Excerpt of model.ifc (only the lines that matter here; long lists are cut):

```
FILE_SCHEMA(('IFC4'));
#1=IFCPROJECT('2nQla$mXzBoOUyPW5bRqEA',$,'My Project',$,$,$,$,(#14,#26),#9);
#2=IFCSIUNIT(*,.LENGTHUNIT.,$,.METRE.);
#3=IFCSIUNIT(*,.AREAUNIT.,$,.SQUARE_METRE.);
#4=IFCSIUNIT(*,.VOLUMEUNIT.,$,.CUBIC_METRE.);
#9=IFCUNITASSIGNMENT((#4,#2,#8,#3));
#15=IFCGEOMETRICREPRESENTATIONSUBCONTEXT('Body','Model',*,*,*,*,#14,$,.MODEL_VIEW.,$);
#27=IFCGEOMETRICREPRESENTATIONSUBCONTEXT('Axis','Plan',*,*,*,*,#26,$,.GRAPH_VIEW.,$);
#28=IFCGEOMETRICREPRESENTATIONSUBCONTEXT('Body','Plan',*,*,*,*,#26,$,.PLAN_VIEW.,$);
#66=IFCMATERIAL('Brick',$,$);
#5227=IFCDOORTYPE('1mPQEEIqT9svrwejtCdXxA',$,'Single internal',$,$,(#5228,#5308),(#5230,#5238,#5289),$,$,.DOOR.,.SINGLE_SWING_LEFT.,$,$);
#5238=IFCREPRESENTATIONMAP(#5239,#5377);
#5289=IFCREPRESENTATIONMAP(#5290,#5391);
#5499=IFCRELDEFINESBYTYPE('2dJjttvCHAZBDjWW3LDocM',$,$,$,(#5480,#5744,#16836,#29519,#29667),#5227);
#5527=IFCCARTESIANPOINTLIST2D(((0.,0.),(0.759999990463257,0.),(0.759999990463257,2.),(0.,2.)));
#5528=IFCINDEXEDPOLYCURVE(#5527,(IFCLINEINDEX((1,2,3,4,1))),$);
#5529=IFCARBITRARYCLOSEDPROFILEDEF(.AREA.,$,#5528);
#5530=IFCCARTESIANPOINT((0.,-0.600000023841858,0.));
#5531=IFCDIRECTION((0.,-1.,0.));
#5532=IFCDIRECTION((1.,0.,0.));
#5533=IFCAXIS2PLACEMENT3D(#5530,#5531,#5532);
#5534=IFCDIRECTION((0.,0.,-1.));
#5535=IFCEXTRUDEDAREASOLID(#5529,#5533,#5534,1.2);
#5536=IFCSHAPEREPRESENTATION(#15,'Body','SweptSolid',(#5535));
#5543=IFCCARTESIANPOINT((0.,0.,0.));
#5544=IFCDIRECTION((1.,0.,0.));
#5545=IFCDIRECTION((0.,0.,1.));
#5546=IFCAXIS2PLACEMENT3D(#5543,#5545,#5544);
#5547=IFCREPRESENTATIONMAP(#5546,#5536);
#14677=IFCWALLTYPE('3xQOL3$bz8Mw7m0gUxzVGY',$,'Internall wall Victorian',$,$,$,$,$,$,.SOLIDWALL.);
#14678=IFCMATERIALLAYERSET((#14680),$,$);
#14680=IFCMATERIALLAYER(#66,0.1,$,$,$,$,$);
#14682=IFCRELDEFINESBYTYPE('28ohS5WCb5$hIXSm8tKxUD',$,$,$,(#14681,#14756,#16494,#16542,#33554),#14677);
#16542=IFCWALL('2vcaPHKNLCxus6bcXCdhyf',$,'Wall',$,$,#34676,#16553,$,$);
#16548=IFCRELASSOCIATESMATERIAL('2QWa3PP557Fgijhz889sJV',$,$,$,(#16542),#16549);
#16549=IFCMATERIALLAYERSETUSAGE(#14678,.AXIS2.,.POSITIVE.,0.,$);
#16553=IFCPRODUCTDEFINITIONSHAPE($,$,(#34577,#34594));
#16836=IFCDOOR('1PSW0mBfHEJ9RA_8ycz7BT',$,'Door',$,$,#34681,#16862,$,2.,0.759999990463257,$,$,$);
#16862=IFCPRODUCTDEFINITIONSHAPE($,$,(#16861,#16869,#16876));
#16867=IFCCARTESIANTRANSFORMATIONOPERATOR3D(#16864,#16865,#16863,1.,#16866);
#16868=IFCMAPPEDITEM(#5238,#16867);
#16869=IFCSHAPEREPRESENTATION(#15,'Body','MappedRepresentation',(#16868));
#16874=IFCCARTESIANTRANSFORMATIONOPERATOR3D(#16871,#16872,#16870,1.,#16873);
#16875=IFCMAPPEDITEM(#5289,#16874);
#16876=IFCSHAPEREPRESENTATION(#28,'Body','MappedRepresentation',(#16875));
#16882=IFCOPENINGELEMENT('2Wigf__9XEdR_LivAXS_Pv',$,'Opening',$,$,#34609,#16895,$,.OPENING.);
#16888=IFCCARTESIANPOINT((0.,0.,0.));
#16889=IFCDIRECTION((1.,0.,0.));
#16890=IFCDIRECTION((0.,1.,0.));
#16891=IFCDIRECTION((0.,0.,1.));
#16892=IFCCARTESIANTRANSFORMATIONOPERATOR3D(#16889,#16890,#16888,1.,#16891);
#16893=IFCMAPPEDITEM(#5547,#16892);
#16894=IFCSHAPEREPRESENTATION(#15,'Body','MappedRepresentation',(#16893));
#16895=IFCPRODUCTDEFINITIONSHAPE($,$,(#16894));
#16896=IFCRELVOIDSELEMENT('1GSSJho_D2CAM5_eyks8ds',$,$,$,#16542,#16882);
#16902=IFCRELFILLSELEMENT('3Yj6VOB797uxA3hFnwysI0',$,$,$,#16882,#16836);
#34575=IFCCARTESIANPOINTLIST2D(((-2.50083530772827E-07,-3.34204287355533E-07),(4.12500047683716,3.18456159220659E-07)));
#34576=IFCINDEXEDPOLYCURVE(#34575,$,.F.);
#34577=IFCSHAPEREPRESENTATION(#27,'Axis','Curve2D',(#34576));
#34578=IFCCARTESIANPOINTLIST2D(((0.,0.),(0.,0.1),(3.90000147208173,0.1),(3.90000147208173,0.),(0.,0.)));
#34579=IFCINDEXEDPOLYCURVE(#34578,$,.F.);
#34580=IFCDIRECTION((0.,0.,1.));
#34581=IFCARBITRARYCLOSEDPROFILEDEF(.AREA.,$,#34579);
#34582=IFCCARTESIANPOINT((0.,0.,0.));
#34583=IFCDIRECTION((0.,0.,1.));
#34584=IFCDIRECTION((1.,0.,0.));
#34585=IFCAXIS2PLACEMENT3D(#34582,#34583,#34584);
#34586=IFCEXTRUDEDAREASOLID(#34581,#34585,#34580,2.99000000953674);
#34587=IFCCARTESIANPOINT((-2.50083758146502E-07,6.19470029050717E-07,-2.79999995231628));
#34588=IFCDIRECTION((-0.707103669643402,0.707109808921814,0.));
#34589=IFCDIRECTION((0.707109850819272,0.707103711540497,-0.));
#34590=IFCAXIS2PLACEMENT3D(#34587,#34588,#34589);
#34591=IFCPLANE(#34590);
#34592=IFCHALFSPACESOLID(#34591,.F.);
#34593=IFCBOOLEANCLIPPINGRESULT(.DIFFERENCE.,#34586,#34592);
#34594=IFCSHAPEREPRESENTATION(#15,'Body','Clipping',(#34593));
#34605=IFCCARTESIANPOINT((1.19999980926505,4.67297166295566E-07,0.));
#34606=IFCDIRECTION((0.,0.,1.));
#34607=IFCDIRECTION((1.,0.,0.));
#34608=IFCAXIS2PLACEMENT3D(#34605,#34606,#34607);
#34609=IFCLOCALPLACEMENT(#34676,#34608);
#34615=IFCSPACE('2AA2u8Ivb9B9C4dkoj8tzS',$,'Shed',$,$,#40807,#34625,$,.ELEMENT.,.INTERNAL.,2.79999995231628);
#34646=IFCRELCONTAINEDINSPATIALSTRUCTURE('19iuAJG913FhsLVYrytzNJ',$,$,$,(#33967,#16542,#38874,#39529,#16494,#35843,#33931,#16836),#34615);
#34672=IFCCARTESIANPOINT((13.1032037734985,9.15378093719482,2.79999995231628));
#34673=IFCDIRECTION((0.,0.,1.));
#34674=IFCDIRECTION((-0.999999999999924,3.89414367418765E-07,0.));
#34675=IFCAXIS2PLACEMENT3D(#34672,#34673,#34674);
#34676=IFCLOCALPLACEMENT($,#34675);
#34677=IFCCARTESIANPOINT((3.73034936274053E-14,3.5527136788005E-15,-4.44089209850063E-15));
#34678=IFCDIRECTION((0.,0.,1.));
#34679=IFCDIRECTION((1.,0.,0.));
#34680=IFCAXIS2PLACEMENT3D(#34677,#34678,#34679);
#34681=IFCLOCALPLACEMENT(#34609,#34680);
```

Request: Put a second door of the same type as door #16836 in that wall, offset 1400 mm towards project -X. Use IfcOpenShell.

```python
import ifcopenshell
import ifcopenshell.api.feature
import ifcopenshell.api.geometry
import ifcopenshell.api.root
import ifcopenshell.geom
import ifcopenshell.util.element
import ifcopenshell.util.placement
import ifcopenshell.util.shape
import ifcopenshell.util.unit

model = ifcopenshell.open("model.ifc")
unit_scale = ifcopenshell.util.unit.calculate_unit_scale(model)
settings = ifcopenshell.geom.settings()


def volume(element):
    """Net volume in cubic metres, openings subtracted."""
    shape = ifcopenshell.geom.create_shape(settings, element)
    return ifcopenshell.util.shape.get_volume(shape.geometry)


door = model.by_id(16836)
opening = door.FillsVoids[0].RelatingOpeningElement
wall = opening.VoidsElements[0].RelatingBuildingElement
before = volume(wall)
shift = ifcopenshell.util.placement.get_local_placement(wall.ObjectPlacement)[:3, 0] * 1.4 / unit_scale

# copy_class copies the void relationship, type, container and properties, but no geometry.
new_opening = ifcopenshell.api.root.copy_class(model, product=opening)
new_opening.Representation = ifcopenshell.util.element.copy_deep(
    model, opening.Representation, exclude=["IfcGeometricRepresentationContext", "IfcRepresentationMap"]
)
new_door = ifcopenshell.api.root.copy_class(model, product=door)
new_door.Representation = ifcopenshell.util.element.copy_deep(
    model, door.Representation, exclude=["IfcGeometricRepresentationContext", "IfcRepresentationMap"]
)
ifcopenshell.api.feature.add_filling(model, opening=new_opening, element=new_door)

for old, new in ((opening, new_opening), (door, new_door)):
    matrix = ifcopenshell.util.placement.get_local_placement(old.ObjectPlacement)
    matrix[:3, 3] += shift
    ifcopenshell.api.geometry.edit_object_placement(model, product=new, matrix=matrix, is_si=False)

after = volume(wall)

print(f"wall volume {before:.3f} -> {after:.3f} m3")

model.write("model_edited.ifc")
```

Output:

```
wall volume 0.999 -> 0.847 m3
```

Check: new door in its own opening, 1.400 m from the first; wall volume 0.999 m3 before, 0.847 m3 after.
